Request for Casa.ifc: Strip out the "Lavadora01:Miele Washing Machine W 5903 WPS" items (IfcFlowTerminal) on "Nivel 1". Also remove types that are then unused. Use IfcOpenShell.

First a look at what the model holds.

```python
import ifcopenshell
import ifcopenshell.util.element

model = ifcopenshell.open("Casa.ifc")
print(model.schema)
storey = next(s for s in model.by_type("IfcBuildingStorey") if s.Name == "Nivel 1")
terminals = [e for e in ifcopenshell.util.element.get_decomposition(storey) if e.is_a("IfcFlowTerminal")]
seen = {}
for e in terminals:
    element_type = ifcopenshell.util.element.get_type(e)
    name = element_type.Name if element_type not in (None, e) else None
    seen[name] = seen.get(name, 0) + 1
for name, count in sorted(seen.items(), key=str):
    print(count, "x", name)
```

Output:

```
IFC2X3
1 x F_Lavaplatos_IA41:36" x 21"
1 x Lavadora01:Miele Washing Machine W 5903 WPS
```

```python
import ifcopenshell
import ifcopenshell.api.root
import ifcopenshell.util.element

model = ifcopenshell.open("Casa.ifc")

storey = next(s for s in model.by_type("IfcBuildingStorey") if s.Name == "Nivel 1")
terminals = [e for e in ifcopenshell.util.element.get_decomposition(storey) if e.is_a("IfcFlowTerminal")]
targets = [e for e in terminals if (t := ifcopenshell.util.element.get_type(e)) not in (None, e) and t.Name == "Lavadora01:Miele Washing Machine W 5903 WPS"]
types = {ifcopenshell.util.element.get_type(e) for e in targets} - {None, *targets}

for e in targets:
    ifcopenshell.api.root.remove_product(model, product=e)
print(len(targets), "removed")

unused = [t for t in types if not ifcopenshell.util.element.get_types(t)]
for t in unused:
    ifcopenshell.api.root.remove_product(model, product=t)
print(len(unused), "unused types removed")

model.write("Casa-out.ifc")
```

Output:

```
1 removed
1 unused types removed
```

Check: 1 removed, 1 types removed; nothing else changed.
